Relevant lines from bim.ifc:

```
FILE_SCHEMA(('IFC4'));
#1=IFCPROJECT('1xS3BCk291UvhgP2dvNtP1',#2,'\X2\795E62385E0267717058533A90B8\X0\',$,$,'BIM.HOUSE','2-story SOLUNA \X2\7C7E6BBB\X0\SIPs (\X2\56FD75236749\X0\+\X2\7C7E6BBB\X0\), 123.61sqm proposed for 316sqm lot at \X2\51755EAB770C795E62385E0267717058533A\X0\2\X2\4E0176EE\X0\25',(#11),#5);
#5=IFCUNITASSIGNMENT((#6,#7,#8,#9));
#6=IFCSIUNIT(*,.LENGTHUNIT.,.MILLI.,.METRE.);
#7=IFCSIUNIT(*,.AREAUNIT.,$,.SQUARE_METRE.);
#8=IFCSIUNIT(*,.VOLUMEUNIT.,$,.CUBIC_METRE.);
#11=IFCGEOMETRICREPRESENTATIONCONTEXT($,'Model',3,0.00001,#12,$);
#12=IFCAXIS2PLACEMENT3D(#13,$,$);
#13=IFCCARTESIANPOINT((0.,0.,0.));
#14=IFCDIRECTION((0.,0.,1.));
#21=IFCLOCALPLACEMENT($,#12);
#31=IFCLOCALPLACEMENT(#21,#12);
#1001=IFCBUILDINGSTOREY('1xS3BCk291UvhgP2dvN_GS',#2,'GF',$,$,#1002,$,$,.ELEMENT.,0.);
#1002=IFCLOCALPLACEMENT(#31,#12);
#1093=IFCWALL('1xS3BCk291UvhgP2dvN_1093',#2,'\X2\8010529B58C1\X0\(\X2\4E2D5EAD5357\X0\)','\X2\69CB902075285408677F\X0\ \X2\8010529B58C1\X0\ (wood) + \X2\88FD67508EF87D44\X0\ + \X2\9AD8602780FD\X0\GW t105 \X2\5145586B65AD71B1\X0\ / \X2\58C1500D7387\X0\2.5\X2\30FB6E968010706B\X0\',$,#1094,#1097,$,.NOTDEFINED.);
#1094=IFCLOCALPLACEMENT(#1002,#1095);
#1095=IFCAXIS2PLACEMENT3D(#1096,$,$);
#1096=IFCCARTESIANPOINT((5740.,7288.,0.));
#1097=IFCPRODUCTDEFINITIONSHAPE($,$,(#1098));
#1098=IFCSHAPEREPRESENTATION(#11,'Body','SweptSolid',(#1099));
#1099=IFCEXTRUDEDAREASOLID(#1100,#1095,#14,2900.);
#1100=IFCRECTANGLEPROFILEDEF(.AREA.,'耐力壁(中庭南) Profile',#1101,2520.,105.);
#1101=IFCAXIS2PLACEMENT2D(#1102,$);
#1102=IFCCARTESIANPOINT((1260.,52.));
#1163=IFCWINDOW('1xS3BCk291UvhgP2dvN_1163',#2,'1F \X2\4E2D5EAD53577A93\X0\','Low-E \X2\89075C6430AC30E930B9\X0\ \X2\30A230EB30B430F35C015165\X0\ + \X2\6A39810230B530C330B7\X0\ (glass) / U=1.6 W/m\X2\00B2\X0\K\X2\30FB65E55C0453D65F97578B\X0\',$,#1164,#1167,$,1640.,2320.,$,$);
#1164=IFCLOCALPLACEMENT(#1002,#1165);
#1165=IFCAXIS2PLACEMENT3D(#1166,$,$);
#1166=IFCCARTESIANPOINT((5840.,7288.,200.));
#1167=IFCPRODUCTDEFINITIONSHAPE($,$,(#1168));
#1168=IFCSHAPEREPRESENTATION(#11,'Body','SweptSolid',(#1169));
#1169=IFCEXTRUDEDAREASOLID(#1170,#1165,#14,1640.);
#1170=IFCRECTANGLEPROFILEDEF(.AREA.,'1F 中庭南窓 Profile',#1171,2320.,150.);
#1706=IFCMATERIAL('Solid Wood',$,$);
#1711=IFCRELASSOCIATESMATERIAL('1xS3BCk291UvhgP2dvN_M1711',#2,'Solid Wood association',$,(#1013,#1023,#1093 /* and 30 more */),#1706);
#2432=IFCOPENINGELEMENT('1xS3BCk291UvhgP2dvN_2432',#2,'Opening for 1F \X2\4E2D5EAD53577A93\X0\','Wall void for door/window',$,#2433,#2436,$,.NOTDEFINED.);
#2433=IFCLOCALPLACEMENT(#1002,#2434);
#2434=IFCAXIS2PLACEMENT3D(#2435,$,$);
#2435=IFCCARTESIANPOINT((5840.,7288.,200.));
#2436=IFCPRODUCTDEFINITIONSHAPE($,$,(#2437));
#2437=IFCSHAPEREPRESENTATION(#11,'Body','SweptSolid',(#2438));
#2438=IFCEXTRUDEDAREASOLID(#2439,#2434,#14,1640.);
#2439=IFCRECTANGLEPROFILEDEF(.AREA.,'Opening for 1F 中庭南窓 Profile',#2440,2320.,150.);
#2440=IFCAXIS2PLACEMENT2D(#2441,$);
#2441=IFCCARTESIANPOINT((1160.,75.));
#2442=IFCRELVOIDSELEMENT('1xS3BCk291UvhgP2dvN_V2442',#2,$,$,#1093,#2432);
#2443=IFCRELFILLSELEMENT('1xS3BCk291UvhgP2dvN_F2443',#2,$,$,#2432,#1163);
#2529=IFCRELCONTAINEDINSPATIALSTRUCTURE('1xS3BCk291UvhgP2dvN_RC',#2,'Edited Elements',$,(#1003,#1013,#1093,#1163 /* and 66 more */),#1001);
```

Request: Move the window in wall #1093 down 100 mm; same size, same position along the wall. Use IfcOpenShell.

```python
import numpy as np
import ifcopenshell
import ifcopenshell.api.geometry
import ifcopenshell.util.placement
import ifcopenshell.util.unit

model = ifcopenshell.open("bim.ifc")
unit_scale = ifcopenshell.util.unit.calculate_unit_scale(model)

window = model.by_guid("1xS3BCk291UvhgP2dvN_1163")
opening = window.FillsVoids[0].RelatingOpeningElement
dz = -0.1 / unit_scale

shift = np.array([0.0, 0.0, dz])
# The window is not placed relative to its opening, so move both.
for product in (opening, window):
    matrix = ifcopenshell.util.placement.get_local_placement(product.ObjectPlacement)
    matrix[:3, 3] += shift
    ifcopenshell.api.geometry.edit_object_placement(model, product=product, matrix=matrix, is_si=False)

print(f"moved by {dz * unit_scale:+.3f} m")

model.write("bim-out.ifc")
```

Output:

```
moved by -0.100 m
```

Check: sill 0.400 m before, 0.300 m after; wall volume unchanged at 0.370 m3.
